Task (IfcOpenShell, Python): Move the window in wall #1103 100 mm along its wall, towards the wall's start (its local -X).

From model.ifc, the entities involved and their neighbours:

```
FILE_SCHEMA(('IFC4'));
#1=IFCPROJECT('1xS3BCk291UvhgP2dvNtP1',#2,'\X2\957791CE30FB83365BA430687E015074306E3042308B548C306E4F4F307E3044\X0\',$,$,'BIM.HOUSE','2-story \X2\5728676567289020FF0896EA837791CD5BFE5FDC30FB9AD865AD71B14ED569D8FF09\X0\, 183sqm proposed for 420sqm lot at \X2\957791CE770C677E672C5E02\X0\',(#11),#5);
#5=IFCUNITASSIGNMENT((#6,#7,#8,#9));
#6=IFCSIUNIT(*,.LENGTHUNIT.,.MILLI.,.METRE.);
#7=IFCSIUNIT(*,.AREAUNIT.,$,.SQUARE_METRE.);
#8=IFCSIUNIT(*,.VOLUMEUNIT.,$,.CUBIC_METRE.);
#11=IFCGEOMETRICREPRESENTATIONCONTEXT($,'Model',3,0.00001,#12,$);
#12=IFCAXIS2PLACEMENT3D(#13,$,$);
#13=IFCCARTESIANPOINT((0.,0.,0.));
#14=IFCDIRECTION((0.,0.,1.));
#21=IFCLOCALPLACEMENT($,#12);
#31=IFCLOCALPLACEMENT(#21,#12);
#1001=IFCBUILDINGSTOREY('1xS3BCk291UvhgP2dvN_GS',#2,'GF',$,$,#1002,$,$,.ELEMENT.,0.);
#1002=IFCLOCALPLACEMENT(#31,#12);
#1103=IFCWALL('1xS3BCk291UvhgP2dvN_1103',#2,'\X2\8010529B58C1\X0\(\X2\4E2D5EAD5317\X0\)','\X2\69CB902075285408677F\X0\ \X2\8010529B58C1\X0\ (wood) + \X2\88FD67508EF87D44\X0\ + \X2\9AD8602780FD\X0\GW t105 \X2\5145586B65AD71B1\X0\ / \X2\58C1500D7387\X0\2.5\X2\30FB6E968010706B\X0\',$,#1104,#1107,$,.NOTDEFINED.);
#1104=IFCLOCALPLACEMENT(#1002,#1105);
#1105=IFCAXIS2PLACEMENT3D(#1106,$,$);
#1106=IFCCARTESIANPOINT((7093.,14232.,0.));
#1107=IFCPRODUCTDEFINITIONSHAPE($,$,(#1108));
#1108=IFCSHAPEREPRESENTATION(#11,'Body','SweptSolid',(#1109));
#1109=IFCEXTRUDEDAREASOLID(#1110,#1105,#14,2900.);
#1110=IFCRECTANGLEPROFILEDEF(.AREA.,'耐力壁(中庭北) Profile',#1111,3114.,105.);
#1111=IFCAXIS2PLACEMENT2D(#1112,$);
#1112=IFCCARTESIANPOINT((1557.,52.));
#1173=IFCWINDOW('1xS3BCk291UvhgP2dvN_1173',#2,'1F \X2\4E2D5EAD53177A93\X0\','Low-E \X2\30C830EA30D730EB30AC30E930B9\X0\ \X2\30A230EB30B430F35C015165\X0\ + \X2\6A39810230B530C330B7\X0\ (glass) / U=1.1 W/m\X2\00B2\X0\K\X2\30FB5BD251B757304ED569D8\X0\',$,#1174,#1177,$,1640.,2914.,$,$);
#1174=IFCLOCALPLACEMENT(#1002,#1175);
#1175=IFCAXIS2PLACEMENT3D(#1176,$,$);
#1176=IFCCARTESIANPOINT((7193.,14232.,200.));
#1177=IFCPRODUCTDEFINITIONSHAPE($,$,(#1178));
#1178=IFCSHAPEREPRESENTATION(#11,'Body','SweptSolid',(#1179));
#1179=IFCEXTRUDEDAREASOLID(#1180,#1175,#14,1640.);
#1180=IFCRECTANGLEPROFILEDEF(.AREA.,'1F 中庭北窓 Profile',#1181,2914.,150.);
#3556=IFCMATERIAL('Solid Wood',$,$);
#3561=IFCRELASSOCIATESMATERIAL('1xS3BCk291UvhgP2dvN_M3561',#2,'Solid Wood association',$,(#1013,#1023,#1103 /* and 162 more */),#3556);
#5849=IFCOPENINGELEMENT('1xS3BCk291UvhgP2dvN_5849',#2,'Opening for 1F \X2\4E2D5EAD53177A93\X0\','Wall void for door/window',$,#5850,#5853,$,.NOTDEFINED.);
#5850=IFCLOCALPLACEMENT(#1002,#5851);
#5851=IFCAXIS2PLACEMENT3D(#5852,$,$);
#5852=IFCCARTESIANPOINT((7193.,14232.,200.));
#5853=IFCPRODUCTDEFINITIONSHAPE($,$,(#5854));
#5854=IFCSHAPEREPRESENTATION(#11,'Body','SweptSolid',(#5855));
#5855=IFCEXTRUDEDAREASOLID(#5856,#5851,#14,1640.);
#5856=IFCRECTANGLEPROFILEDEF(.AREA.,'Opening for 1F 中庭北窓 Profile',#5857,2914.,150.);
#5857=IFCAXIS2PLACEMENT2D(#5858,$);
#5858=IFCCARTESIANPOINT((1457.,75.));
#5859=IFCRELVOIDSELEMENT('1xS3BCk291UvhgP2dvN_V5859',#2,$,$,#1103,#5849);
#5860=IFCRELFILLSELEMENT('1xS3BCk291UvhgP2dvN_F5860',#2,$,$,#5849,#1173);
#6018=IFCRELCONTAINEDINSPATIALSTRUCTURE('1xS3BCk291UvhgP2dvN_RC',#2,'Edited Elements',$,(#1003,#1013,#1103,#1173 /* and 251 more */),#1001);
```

```python
import ifcopenshell
import ifcopenshell.api.geometry
import ifcopenshell.util.placement
import ifcopenshell.util.unit

model = ifcopenshell.open("model.ifc")
unit_scale = ifcopenshell.util.unit.calculate_unit_scale(model)

window = model.by_guid("1xS3BCk291UvhgP2dvN_1173")
opening = window.FillsVoids[0].RelatingOpeningElement
wall = opening.VoidsElements[0].RelatingBuildingElement

wall_matrix = ifcopenshell.util.placement.get_local_placement(wall.ObjectPlacement)
shift = wall_matrix[:3, 0] * -0.1 / unit_scale
before = ifcopenshell.util.placement.get_local_placement(window.ObjectPlacement)[:3, 3].copy()

# The window is not placed relative to its opening, so move both.
for product in (opening, window):
    matrix = ifcopenshell.util.placement.get_local_placement(product.ObjectPlacement)
    matrix[:3, 3] += shift
    ifcopenshell.api.geometry.edit_object_placement(model, product=product, matrix=matrix, is_si=False)

after = ifcopenshell.util.placement.get_local_placement(window.ObjectPlacement)[:3, 3]
print("window moved by", (after - before).round(3) + 0.0)

model.write("model_edited.ifc")
```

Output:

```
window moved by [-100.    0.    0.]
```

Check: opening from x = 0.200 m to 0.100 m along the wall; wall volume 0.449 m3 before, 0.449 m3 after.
